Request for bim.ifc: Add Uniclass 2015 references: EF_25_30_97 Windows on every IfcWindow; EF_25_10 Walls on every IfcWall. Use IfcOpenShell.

First a look at what the model holds.

```python
import ifcopenshell

model = ifcopenshell.open("bim.ifc")
print(model.schema)
print("classifications:", [c.Name for c in model.by_type("IfcClassification")])
for ifc_class in ("IfcDoor", "IfcRoof", "IfcStair", "IfcWall", "IfcWindow"):
    print(ifc_class, len(model.by_type(ifc_class)))
```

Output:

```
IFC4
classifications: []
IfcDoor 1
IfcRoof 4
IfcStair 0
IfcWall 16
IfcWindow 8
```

```python
import ifcopenshell
import ifcopenshell.api.classification

model = ifcopenshell.open("bim.ifc")

system = ifcopenshell.api.classification.add_classification(model, classification="Uniclass 2015")

codes = {
    "IfcWindow": ("EF_25_30_97", "Windows"),
    "IfcWall": ("EF_25_10", "Walls"),
}
for ifc_class, (code, name) in codes.items():
    products = model.by_type(ifc_class)
    ifcopenshell.api.classification.add_reference(
        model, products=products, classification=system, identification=code, name=name
    )
    print(code, len(products))

model.write("bim_edited.ifc")
```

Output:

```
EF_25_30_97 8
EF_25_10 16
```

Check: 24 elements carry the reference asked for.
